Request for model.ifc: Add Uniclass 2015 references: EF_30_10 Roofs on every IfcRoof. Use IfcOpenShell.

First a look at what the model holds.

```python
import ifcopenshell

model = ifcopenshell.open("model.ifc")
print(model.schema)
print("classifications:", [c.Name for c in model.by_type("IfcClassification")])
for ifc_class in ("IfcDoor", "IfcRoof", "IfcStair", "IfcWall", "IfcWindow"):
    print(ifc_class, len(model.by_type(ifc_class)))
```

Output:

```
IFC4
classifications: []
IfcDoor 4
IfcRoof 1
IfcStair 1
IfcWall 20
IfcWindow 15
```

```python
import ifcopenshell
import ifcopenshell.api.classification

model = ifcopenshell.open("model.ifc")

system = ifcopenshell.api.classification.add_classification(model, classification="Uniclass 2015")

codes = {
    "IfcRoof": ("EF_30_10", "Roofs"),
}
for ifc_class, (code, name) in codes.items():
    products = model.by_type(ifc_class)
    ifcopenshell.api.classification.add_reference(
        model, products=products, classification=system, identification=code, name=name
    )
    print(code, len(products))

model.write("model-out.ifc")
```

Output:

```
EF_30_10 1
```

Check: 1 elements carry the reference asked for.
